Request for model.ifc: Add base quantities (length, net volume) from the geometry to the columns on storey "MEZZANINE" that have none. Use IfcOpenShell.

First a look at what the model holds.

```python
import ifcopenshell
import ifcopenshell.util.element
import ifcopenshell.util.unit

model = ifcopenshell.open("model.ifc")
print(model.schema)
for unit_type in ("LENGTHUNIT", "AREAUNIT", "VOLUMEUNIT"):
    print(unit_type, ifcopenshell.util.unit.calculate_unit_scale(model, unit_type))
storey = next(s for s in model.by_type("IfcBuildingStorey") if s.Name == "MEZZANINE")
columns = [e for e in ifcopenshell.util.element.get_decomposition(storey) if e.is_a("IfcColumn")]
for e in sorted(columns, key=lambda e: e.id()):
    print(e.id(), e.is_a(), e.Name, list(ifcopenshell.util.element.get_psets(e, qtos_only=True)), sep=" | ")
```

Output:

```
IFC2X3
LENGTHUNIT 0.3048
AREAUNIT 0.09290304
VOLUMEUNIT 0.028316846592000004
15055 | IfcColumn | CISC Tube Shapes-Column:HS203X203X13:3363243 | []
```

```python
import ifcopenshell
import ifcopenshell.api.pset
import ifcopenshell.geom
import ifcopenshell.util.element
import ifcopenshell.util.shape
import ifcopenshell.util.unit

model = ifcopenshell.open("model.ifc")
unit_scale = ifcopenshell.util.unit.calculate_unit_scale(model)
volume_scale = ifcopenshell.util.unit.calculate_unit_scale(model, "VOLUMEUNIT")
settings = ifcopenshell.geom.settings()

storey = next(s for s in model.by_type("IfcBuildingStorey") if s.Name == "MEZZANINE")
columns = [e for e in ifcopenshell.util.element.get_decomposition(storey) if e.is_a("IfcColumn")]

for e in sorted(columns, key=lambda e: e.id()):
    if ifcopenshell.util.element.get_psets(e, qtos_only=True, should_inherit=False):
        continue
    # Geometry comes back in metres, in the element's own axes.
    shape = ifcopenshell.geom.create_shape(settings, e)
    values = {
        "Length": ifcopenshell.util.shape.get_z(shape.geometry) / unit_scale,
        "NetVolume": ifcopenshell.util.shape.get_volume(shape.geometry) / volume_scale,
    }
    qto = ifcopenshell.api.pset.add_qto(model, product=e, name="BaseQuantities")
    ifcopenshell.api.pset.edit_qto(model, qto=qto, properties=values)
    print(e.id(), {k: round(v, 3) for k, v in values.items()})

model.write("model_edited.ifc")
```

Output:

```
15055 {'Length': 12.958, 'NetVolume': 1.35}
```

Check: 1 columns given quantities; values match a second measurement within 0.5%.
